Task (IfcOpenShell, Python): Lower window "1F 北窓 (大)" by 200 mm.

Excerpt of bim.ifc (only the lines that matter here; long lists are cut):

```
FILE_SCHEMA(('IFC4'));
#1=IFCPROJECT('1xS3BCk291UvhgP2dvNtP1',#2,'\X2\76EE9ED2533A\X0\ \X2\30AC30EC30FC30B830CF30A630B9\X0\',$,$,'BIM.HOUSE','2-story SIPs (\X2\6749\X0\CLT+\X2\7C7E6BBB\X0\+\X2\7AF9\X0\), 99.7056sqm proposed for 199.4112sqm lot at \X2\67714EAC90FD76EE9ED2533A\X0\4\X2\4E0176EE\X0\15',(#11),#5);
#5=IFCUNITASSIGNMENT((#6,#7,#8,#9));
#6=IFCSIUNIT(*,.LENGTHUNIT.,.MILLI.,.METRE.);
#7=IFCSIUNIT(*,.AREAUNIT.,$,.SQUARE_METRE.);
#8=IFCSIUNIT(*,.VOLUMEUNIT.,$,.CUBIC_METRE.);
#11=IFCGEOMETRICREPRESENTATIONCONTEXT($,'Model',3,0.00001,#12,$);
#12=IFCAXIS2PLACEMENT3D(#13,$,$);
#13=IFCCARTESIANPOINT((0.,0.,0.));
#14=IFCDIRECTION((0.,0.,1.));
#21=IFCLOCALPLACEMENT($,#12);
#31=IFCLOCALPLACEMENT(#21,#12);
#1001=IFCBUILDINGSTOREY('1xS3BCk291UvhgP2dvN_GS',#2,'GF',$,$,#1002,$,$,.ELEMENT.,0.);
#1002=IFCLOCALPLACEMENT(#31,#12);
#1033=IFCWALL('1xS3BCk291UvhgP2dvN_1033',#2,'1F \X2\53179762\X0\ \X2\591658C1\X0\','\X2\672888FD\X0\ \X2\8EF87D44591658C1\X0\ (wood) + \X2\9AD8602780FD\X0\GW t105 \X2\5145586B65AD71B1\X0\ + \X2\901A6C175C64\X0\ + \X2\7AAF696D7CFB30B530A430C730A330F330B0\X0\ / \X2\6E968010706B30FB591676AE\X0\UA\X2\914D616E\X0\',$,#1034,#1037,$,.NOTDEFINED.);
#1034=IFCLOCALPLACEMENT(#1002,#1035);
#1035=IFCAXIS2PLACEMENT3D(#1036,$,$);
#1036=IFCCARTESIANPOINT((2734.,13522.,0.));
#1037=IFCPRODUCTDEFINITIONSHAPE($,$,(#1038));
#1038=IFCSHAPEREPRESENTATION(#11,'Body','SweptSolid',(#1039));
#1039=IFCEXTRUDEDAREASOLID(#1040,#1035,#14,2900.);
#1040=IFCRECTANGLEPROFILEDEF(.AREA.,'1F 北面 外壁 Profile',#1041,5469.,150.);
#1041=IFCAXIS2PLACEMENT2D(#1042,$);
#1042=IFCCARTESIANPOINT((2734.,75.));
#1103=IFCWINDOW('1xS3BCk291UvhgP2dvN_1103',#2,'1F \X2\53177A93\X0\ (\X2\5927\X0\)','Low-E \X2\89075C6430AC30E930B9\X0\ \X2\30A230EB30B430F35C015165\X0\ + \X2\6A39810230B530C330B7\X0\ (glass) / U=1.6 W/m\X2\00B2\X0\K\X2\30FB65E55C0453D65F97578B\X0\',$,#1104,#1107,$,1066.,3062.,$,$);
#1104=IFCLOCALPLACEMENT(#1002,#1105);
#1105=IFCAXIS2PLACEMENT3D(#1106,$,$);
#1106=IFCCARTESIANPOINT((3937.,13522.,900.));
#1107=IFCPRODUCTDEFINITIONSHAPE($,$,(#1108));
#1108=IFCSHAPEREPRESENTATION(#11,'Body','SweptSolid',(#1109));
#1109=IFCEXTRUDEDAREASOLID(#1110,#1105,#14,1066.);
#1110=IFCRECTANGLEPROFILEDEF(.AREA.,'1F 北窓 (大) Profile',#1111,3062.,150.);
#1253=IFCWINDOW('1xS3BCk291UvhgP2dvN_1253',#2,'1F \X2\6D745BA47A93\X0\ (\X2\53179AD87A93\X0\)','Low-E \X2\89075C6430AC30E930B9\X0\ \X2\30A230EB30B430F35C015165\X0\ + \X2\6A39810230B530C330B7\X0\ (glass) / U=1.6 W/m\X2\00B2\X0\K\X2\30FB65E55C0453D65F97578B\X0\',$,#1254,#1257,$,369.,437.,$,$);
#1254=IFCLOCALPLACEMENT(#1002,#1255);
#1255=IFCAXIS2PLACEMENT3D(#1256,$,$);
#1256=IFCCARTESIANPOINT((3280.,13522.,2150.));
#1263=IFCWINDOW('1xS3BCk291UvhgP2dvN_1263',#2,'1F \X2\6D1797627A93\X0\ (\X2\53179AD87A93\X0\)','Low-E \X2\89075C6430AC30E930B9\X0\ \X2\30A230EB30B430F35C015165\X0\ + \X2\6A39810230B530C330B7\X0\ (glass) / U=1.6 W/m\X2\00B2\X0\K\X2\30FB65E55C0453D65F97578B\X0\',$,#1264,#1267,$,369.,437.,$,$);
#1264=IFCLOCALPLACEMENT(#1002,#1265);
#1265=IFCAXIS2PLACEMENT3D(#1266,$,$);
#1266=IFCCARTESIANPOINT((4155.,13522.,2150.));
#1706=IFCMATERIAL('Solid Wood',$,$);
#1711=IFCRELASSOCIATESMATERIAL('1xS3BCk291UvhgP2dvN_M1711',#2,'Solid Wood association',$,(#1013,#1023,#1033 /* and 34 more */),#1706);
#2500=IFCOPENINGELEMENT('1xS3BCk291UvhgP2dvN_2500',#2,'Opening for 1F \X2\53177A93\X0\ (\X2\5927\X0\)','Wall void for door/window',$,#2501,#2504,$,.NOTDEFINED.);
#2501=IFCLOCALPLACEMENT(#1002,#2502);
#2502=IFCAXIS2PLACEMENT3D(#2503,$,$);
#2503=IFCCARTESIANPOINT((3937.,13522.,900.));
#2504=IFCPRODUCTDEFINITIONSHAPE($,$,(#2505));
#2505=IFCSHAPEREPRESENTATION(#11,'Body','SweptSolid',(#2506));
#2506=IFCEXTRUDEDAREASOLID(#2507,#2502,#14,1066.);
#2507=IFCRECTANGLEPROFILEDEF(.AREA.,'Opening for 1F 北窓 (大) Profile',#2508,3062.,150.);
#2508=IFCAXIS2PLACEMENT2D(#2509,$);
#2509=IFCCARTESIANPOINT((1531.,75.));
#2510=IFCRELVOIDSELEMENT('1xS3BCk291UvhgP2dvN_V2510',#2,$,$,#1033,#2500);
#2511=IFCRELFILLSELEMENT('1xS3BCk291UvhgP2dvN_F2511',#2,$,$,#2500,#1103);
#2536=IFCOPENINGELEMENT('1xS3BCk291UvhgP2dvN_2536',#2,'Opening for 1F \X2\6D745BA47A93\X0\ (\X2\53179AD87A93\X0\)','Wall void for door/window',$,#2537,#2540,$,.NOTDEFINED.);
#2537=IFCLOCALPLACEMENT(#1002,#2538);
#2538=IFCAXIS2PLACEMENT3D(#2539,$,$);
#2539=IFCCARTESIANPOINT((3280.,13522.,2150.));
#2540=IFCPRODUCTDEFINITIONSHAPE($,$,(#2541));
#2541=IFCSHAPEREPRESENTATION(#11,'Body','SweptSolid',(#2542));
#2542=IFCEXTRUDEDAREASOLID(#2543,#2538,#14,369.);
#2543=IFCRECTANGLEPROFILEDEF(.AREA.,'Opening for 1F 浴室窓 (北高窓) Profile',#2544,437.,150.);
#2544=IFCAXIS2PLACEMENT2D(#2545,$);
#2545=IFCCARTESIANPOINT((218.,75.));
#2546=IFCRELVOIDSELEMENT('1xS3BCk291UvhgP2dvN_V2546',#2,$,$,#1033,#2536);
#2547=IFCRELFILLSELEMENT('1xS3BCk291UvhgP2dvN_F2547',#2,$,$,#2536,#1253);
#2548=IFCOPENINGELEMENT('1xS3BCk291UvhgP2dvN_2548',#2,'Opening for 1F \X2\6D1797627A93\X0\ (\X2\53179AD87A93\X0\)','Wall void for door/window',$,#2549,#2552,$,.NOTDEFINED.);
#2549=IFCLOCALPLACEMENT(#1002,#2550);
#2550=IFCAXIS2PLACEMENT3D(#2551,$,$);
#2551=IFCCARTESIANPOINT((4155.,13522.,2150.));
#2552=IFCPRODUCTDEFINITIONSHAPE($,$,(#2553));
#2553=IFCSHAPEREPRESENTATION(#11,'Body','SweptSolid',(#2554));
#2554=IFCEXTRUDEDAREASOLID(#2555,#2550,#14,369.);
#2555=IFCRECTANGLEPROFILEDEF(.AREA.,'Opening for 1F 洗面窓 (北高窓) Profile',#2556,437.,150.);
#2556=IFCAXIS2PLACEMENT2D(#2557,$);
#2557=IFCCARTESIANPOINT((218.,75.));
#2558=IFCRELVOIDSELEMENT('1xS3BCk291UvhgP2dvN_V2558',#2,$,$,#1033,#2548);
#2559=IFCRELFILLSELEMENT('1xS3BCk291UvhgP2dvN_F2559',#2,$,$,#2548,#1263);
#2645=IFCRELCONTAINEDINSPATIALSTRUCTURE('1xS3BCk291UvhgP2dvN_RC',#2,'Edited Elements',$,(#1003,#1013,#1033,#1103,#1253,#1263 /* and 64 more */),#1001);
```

```python
import numpy as np
import ifcopenshell
import ifcopenshell.api.geometry
import ifcopenshell.util.placement
import ifcopenshell.util.unit

model = ifcopenshell.open("bim.ifc")
unit_scale = ifcopenshell.util.unit.calculate_unit_scale(model)

window = model.by_guid("1xS3BCk291UvhgP2dvN_1103")
opening = window.FillsVoids[0].RelatingOpeningElement
dz = -200.0

shift = np.array([0.0, 0.0, dz])
# The window is not placed relative to its opening, so move both.
for product in (opening, window):
    matrix = ifcopenshell.util.placement.get_local_placement(product.ObjectPlacement)
    matrix[:3, 3] += shift
    ifcopenshell.api.geometry.edit_object_placement(model, product=product, matrix=matrix, is_si=False)

print(f"moved by {dz * unit_scale:+.3f} m")

model.write("bim_rev.ifc")
```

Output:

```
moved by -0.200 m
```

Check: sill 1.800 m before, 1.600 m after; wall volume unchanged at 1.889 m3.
